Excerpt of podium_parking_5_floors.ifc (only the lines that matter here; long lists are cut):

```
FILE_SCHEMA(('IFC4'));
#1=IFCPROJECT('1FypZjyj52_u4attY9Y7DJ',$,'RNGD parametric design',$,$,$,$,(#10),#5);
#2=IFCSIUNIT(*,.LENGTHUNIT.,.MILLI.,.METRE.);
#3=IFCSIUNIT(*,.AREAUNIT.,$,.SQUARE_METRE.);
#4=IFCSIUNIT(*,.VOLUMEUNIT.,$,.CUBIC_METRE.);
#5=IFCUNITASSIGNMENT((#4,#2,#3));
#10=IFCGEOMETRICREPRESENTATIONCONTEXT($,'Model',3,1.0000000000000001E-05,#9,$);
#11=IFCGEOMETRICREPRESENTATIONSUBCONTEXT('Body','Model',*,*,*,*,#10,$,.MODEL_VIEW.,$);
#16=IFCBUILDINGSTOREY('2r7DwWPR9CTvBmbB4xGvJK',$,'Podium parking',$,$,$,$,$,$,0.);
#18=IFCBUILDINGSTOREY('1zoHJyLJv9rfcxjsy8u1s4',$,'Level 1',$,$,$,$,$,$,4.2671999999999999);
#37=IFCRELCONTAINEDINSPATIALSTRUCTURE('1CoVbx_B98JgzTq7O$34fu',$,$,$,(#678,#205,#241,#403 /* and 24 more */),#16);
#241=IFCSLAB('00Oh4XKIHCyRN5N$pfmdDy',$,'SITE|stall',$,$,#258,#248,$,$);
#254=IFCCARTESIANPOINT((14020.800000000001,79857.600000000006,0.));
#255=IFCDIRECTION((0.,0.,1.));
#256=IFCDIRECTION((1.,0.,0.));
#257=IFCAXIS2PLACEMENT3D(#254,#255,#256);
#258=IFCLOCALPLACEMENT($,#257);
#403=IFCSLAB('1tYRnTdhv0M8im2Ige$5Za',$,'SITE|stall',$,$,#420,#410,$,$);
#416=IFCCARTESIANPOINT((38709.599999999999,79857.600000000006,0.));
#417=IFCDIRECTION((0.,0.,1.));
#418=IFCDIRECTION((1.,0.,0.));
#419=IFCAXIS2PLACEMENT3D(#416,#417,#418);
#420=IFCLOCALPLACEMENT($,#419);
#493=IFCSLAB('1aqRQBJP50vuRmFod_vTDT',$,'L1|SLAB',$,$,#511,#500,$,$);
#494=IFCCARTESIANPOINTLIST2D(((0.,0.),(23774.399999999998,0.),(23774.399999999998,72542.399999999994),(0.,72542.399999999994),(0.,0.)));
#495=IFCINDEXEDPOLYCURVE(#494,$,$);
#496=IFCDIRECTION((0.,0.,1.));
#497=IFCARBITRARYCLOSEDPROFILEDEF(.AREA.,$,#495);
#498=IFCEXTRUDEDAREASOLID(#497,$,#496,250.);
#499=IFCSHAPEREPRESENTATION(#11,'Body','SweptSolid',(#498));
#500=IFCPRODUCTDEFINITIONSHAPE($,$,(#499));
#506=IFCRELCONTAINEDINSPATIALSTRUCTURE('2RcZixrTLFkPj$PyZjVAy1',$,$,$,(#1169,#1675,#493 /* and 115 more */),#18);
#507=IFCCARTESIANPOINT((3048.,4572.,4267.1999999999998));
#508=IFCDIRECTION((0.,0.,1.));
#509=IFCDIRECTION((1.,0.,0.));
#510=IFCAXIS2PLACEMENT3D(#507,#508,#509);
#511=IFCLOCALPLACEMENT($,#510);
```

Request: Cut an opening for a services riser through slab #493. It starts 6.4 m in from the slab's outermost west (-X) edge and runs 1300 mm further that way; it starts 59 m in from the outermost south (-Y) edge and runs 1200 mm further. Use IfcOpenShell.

```python
import numpy as np
import ifcopenshell
import ifcopenshell.api.feature
import ifcopenshell.api.geometry
import ifcopenshell.api.root
import ifcopenshell.geom
import ifcopenshell.util.placement
import ifcopenshell.util.representation
import ifcopenshell.util.shape
import ifcopenshell.util.unit

model = ifcopenshell.open("podium_parking_5_floors.ifc")
unit_scale = ifcopenshell.util.unit.calculate_unit_scale(model)
settings = ifcopenshell.geom.settings()


def volume(element):
    """Net volume in cubic metres, openings subtracted."""
    shape = ifcopenshell.geom.create_shape(settings, element)
    return ifcopenshell.util.shape.get_volume(shape.geometry)


slab = model.by_guid("1aqRQBJP50vuRmFod_vTDT")
before = volume(slab)

# Extent in the slab's own axes, in metres. The edges named are its -X and -Y sides.
slab_shape = ifcopenshell.geom.create_shape(settings, slab)
vertices = ifcopenshell.util.shape.get_vertices(slab_shape.geometry)
x_min, y_min, bottom = vertices.min(axis=0)
top = vertices[:, 2].max()

opening = ifcopenshell.api.root.create_entity(model, ifc_class="IfcOpeningElement", name="Services riser opening", predefined_type="OPENING")
context = ifcopenshell.util.representation.get_context(model, "Model", "Body", "MODEL_VIEW")
width, depth = 1.3, 1.2
outline = [(0.0, 0.0), (width, 0.0), (width, depth), (0.0, depth), (0.0, 0.0)]
# Overshoot both faces by 50 mm so the cut is clean.
shape = ifcopenshell.api.geometry.add_slab_representation(
    model, context=context, depth=top - bottom + 0.1, polyline=outline
)
ifcopenshell.api.geometry.assign_representation(model, product=opening, representation=shape)

matrix = ifcopenshell.util.placement.get_local_placement(slab.ObjectPlacement)
matrix[:, 3] = matrix @ np.append(np.array([x_min + 6.4, y_min + 59, bottom - 0.05]) / unit_scale, 1.0)
ifcopenshell.api.geometry.edit_object_placement(model, product=opening, matrix=matrix, is_si=False)
ifcopenshell.api.feature.add_feature(model, feature=opening, element=slab)

after = volume(slab)

print(f"slab volume {before:.3f} -> {after:.3f} m3")

model.write("podium_parking_5_floors_edited.ifc")
```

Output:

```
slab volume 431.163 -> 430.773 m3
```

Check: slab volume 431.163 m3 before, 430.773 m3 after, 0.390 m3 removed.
